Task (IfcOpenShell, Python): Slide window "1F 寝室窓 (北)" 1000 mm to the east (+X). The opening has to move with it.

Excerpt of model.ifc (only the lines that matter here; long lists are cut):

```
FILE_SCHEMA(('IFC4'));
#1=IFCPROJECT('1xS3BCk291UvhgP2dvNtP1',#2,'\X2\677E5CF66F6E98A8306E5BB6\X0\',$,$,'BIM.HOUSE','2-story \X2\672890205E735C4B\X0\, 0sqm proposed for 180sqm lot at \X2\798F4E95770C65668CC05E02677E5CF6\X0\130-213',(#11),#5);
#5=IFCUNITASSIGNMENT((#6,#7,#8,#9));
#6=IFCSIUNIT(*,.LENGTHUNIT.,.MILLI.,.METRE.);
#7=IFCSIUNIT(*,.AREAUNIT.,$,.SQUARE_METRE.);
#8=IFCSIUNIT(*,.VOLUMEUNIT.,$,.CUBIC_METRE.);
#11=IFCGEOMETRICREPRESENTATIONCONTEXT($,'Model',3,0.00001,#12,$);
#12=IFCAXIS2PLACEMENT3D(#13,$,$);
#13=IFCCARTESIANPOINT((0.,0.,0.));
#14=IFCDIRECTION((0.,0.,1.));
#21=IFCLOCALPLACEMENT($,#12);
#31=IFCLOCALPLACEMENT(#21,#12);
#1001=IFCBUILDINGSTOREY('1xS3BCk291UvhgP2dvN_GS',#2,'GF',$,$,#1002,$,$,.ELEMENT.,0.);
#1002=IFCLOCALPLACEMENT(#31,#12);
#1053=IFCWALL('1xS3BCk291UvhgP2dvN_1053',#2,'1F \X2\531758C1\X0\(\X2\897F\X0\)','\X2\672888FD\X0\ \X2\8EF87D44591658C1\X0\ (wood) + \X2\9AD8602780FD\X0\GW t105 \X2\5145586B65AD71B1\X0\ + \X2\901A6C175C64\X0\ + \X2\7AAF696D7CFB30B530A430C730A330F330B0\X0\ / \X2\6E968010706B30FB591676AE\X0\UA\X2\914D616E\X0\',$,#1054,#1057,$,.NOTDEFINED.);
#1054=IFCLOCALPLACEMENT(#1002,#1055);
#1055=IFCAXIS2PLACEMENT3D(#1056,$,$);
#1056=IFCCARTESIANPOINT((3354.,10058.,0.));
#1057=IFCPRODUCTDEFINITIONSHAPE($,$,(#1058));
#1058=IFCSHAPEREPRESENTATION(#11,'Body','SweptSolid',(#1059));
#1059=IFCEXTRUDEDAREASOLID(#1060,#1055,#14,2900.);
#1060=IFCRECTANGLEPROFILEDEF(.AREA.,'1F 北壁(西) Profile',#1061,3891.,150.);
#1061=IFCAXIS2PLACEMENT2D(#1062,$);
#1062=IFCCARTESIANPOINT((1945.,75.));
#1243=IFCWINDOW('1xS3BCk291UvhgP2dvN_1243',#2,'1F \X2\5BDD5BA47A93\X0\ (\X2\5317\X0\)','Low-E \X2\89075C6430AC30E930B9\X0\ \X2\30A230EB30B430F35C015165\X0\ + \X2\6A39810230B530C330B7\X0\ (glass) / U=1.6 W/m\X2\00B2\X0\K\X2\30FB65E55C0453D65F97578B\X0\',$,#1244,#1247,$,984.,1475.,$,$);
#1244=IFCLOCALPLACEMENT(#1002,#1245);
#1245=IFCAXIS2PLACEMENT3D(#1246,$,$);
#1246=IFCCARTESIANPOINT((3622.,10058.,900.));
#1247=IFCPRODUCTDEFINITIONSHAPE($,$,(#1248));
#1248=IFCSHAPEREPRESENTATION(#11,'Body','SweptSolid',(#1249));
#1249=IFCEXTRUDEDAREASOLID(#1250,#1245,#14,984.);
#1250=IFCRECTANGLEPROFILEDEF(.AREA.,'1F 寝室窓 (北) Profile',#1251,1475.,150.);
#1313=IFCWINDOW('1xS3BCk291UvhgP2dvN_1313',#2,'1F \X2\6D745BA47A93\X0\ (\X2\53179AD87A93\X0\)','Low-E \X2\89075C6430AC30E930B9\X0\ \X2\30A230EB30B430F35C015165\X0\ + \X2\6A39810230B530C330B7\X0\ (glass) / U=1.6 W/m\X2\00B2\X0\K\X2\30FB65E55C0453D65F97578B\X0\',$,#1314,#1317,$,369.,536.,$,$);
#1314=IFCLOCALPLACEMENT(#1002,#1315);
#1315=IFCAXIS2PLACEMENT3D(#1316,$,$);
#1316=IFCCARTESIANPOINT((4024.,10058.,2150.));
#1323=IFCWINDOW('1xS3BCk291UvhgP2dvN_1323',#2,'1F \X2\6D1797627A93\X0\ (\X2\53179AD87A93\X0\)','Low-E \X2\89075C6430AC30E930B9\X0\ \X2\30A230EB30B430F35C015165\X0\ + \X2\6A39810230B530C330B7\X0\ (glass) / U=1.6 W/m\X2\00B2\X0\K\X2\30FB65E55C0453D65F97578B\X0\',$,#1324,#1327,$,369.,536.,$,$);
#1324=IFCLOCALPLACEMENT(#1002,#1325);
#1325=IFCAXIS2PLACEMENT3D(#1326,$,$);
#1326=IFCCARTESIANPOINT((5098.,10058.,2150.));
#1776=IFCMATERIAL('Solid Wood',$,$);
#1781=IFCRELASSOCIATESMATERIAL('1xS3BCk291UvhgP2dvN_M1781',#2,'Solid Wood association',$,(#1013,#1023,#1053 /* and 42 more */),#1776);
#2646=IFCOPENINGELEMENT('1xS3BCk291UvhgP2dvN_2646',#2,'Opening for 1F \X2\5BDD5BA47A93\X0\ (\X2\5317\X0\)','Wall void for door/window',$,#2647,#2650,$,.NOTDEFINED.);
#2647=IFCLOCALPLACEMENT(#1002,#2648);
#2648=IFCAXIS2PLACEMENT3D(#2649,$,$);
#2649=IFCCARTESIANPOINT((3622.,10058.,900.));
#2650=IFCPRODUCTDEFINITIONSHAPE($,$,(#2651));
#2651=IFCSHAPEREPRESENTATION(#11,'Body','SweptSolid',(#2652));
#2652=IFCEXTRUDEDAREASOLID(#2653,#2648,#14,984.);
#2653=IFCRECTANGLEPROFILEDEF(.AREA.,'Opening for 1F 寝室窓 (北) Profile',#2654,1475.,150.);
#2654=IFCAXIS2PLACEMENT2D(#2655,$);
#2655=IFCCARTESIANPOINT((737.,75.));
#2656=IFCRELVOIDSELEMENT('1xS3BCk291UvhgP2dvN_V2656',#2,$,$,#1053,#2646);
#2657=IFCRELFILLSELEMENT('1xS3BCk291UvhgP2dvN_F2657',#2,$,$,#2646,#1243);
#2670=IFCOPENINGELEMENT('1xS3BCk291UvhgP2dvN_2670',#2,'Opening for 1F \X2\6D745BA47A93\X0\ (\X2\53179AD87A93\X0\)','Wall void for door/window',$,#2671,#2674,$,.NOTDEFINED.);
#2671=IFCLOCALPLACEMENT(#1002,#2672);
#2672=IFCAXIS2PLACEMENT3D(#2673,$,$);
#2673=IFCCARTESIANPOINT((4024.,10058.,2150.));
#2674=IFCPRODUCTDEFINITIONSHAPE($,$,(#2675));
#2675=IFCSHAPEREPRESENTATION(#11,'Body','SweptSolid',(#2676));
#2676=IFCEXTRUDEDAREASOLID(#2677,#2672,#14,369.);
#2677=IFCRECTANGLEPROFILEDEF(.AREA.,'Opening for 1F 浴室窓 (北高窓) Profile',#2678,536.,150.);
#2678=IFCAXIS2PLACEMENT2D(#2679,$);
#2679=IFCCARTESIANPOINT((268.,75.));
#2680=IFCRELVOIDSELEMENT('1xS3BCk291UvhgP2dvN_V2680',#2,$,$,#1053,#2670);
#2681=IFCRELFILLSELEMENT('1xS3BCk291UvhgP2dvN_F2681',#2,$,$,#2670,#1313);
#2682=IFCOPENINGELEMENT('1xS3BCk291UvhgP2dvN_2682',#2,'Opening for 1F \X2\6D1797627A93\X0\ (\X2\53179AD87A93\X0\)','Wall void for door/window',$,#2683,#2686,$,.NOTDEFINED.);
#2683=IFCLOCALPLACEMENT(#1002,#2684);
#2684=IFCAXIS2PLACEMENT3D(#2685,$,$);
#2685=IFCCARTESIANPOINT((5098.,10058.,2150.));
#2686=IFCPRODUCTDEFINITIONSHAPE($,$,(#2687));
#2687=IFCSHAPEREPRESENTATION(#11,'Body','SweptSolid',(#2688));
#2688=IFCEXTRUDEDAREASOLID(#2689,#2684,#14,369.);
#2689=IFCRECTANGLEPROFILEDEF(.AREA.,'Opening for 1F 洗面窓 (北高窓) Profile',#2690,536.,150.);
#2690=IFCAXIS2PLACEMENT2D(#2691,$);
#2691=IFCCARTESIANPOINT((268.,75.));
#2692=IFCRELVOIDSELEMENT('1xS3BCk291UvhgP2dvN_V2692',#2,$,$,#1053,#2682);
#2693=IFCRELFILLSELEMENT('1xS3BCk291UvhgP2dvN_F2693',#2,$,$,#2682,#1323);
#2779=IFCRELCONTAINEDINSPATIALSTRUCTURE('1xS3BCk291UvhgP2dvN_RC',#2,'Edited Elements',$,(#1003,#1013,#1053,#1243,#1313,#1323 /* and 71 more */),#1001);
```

```python
import ifcopenshell
import ifcopenshell.api.geometry
import ifcopenshell.util.placement
import ifcopenshell.util.unit

model = ifcopenshell.open("model.ifc")
unit_scale = ifcopenshell.util.unit.calculate_unit_scale(model)

window = model.by_id(1243)
opening = window.FillsVoids[0].RelatingOpeningElement
wall = opening.VoidsElements[0].RelatingBuildingElement

wall_matrix = ifcopenshell.util.placement.get_local_placement(wall.ObjectPlacement)
shift = wall_matrix[:3, 0] * 1 / unit_scale
before = ifcopenshell.util.placement.get_local_placement(window.ObjectPlacement)[:3, 3].copy()

# The window is not placed relative to its opening, so move both.
for product in (opening, window):
    matrix = ifcopenshell.util.placement.get_local_placement(product.ObjectPlacement)
    matrix[:3, 3] += shift
    ifcopenshell.api.geometry.edit_object_placement(model, product=product, matrix=matrix, is_si=False)

after = ifcopenshell.util.placement.get_local_placement(window.ObjectPlacement)[:3, 3]
print("window moved by", (after - before).round(3) + 0.0)

model.write("model-out.ifc")
```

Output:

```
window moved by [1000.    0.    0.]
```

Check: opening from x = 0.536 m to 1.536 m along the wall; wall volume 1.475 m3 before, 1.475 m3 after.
